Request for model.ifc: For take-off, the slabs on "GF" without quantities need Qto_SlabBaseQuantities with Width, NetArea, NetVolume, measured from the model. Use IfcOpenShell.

First a look at what the model holds.

```python
import ifcopenshell
import ifcopenshell.util.element
import ifcopenshell.util.unit

model = ifcopenshell.open("model.ifc")
print(model.schema)
for unit_type in ("LENGTHUNIT", "AREAUNIT", "VOLUMEUNIT"):
    print(unit_type, ifcopenshell.util.unit.calculate_unit_scale(model, unit_type))
storey = next(s for s in model.by_type("IfcBuildingStorey") if s.Name == "GF")
slabs = [e for e in ifcopenshell.util.element.get_decomposition(storey) if e.is_a("IfcSlab")]
for e in sorted(slabs, key=lambda e: e.id()):
    print(e.id(), e.is_a(), e.Name, list(ifcopenshell.util.element.get_psets(e, qtos_only=True)), sep=" | ")
```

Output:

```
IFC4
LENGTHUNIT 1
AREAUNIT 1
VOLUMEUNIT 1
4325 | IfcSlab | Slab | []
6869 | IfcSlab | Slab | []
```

```python
import ifcopenshell
import ifcopenshell.api.pset
import ifcopenshell.geom
import ifcopenshell.util.element
import ifcopenshell.util.shape
import ifcopenshell.util.unit

model = ifcopenshell.open("model.ifc")
unit_scale = ifcopenshell.util.unit.calculate_unit_scale(model)
area_scale = ifcopenshell.util.unit.calculate_unit_scale(model, "AREAUNIT")
volume_scale = ifcopenshell.util.unit.calculate_unit_scale(model, "VOLUMEUNIT")
settings = ifcopenshell.geom.settings()

storey = next(s for s in model.by_type("IfcBuildingStorey") if s.Name == "GF")
slabs = [e for e in ifcopenshell.util.element.get_decomposition(storey) if e.is_a("IfcSlab")]

for e in sorted(slabs, key=lambda e: e.id()):
    if ifcopenshell.util.element.get_psets(e, qtos_only=True, should_inherit=False):
        continue
    # Geometry comes back in metres, in the element's own axes.
    shape = ifcopenshell.geom.create_shape(settings, e)
    values = {
        "Width": ifcopenshell.util.shape.get_z(shape.geometry) / unit_scale,
        "NetArea": ifcopenshell.util.shape.get_footprint_area(shape.geometry) / area_scale,
        "NetVolume": ifcopenshell.util.shape.get_volume(shape.geometry) / volume_scale,
    }
    qto = ifcopenshell.api.pset.add_qto(model, product=e, name="Qto_SlabBaseQuantities")
    ifcopenshell.api.pset.edit_qto(model, qto=qto, properties=values)
    print(e.id(), {k: round(v, 3) for k, v in values.items()})

model.write("model-out.ifc")
```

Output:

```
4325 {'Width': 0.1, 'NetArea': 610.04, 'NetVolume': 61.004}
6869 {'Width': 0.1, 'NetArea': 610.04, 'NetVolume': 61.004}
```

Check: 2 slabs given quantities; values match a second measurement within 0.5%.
